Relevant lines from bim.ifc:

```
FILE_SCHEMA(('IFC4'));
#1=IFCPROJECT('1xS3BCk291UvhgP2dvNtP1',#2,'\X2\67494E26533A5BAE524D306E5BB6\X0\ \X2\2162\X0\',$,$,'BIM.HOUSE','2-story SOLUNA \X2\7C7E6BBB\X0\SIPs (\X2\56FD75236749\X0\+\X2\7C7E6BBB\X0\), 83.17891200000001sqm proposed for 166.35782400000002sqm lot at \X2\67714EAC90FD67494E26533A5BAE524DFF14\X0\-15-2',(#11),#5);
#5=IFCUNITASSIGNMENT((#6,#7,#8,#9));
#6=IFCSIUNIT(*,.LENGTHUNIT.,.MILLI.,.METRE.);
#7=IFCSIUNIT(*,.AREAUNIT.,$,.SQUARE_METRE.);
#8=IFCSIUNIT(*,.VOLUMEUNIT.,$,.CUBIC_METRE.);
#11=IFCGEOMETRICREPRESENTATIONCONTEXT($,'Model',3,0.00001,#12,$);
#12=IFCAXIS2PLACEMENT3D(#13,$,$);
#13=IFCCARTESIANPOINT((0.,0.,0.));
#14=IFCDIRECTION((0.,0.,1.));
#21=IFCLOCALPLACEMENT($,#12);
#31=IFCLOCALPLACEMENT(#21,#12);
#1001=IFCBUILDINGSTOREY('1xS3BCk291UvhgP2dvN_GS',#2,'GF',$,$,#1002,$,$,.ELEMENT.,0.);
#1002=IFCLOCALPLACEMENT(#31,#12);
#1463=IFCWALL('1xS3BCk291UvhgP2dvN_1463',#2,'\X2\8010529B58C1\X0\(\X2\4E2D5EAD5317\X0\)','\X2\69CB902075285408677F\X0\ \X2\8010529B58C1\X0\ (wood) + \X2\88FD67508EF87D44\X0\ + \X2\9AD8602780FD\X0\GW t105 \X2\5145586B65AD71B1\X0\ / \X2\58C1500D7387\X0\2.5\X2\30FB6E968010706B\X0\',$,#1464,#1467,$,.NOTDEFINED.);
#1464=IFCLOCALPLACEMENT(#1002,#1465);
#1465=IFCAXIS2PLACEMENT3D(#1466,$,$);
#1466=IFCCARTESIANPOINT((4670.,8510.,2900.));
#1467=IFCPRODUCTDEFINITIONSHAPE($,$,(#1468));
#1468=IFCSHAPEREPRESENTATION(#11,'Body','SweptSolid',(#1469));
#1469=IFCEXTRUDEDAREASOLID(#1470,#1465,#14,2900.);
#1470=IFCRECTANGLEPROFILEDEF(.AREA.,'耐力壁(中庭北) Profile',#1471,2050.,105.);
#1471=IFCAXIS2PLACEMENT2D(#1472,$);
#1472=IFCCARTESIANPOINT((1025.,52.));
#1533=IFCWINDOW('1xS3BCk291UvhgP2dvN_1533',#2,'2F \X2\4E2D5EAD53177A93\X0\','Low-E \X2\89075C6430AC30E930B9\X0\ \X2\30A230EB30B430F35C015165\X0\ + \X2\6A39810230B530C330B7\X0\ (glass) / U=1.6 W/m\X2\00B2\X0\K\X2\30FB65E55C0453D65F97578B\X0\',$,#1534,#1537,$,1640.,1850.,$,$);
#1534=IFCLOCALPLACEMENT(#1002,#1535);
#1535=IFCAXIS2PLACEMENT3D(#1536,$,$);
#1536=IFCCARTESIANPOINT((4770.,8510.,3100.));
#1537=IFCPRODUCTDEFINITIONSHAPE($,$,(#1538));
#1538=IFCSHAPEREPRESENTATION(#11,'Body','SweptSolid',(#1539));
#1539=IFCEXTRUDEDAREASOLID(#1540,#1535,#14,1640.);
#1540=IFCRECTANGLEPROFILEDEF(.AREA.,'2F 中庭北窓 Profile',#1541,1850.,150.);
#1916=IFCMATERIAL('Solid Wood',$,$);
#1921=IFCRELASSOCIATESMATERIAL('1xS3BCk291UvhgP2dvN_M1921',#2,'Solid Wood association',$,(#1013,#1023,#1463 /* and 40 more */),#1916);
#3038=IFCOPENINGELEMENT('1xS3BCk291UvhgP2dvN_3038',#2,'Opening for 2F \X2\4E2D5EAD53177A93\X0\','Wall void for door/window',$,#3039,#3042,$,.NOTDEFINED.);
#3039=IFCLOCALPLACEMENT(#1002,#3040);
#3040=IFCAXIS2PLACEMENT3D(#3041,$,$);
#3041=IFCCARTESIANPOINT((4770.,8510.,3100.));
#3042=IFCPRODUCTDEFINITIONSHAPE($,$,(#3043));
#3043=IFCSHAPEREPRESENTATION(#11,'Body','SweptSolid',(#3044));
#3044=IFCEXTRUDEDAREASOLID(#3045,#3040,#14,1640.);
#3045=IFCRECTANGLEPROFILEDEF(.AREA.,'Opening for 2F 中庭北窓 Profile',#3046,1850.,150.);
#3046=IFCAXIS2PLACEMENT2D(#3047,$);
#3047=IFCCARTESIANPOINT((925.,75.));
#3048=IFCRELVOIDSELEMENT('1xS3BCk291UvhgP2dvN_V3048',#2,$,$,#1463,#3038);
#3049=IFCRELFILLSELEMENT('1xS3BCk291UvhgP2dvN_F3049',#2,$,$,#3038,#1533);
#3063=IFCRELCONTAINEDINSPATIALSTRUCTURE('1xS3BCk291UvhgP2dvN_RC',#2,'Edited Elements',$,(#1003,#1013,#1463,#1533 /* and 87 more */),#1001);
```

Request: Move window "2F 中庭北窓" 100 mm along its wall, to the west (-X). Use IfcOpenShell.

```python
import ifcopenshell
import ifcopenshell.api.geometry
import ifcopenshell.util.placement

model = ifcopenshell.open("bim.ifc")

window = model.by_guid("1xS3BCk291UvhgP2dvN_1533")
opening = window.FillsVoids[0].RelatingOpeningElement
wall = opening.VoidsElements[0].RelatingBuildingElement

wall_matrix = ifcopenshell.util.placement.get_local_placement(wall.ObjectPlacement)
shift = wall_matrix[:3, 0] * -100.0
before = ifcopenshell.util.placement.get_local_placement(window.ObjectPlacement)[:3, 3].copy()

# The window is not placed relative to its opening, so move both.
for product in (opening, window):
    matrix = ifcopenshell.util.placement.get_local_placement(product.ObjectPlacement)
    matrix[:3, 3] += shift
    ifcopenshell.api.geometry.edit_object_placement(model, product=product, matrix=matrix, is_si=False)

after = ifcopenshell.util.placement.get_local_placement(window.ObjectPlacement)[:3, 3]
print("window moved by", (after - before).round(3) + 0.0)

model.write("bim-out.ifc")
```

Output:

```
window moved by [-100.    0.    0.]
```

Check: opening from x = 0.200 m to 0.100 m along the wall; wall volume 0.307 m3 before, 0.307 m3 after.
